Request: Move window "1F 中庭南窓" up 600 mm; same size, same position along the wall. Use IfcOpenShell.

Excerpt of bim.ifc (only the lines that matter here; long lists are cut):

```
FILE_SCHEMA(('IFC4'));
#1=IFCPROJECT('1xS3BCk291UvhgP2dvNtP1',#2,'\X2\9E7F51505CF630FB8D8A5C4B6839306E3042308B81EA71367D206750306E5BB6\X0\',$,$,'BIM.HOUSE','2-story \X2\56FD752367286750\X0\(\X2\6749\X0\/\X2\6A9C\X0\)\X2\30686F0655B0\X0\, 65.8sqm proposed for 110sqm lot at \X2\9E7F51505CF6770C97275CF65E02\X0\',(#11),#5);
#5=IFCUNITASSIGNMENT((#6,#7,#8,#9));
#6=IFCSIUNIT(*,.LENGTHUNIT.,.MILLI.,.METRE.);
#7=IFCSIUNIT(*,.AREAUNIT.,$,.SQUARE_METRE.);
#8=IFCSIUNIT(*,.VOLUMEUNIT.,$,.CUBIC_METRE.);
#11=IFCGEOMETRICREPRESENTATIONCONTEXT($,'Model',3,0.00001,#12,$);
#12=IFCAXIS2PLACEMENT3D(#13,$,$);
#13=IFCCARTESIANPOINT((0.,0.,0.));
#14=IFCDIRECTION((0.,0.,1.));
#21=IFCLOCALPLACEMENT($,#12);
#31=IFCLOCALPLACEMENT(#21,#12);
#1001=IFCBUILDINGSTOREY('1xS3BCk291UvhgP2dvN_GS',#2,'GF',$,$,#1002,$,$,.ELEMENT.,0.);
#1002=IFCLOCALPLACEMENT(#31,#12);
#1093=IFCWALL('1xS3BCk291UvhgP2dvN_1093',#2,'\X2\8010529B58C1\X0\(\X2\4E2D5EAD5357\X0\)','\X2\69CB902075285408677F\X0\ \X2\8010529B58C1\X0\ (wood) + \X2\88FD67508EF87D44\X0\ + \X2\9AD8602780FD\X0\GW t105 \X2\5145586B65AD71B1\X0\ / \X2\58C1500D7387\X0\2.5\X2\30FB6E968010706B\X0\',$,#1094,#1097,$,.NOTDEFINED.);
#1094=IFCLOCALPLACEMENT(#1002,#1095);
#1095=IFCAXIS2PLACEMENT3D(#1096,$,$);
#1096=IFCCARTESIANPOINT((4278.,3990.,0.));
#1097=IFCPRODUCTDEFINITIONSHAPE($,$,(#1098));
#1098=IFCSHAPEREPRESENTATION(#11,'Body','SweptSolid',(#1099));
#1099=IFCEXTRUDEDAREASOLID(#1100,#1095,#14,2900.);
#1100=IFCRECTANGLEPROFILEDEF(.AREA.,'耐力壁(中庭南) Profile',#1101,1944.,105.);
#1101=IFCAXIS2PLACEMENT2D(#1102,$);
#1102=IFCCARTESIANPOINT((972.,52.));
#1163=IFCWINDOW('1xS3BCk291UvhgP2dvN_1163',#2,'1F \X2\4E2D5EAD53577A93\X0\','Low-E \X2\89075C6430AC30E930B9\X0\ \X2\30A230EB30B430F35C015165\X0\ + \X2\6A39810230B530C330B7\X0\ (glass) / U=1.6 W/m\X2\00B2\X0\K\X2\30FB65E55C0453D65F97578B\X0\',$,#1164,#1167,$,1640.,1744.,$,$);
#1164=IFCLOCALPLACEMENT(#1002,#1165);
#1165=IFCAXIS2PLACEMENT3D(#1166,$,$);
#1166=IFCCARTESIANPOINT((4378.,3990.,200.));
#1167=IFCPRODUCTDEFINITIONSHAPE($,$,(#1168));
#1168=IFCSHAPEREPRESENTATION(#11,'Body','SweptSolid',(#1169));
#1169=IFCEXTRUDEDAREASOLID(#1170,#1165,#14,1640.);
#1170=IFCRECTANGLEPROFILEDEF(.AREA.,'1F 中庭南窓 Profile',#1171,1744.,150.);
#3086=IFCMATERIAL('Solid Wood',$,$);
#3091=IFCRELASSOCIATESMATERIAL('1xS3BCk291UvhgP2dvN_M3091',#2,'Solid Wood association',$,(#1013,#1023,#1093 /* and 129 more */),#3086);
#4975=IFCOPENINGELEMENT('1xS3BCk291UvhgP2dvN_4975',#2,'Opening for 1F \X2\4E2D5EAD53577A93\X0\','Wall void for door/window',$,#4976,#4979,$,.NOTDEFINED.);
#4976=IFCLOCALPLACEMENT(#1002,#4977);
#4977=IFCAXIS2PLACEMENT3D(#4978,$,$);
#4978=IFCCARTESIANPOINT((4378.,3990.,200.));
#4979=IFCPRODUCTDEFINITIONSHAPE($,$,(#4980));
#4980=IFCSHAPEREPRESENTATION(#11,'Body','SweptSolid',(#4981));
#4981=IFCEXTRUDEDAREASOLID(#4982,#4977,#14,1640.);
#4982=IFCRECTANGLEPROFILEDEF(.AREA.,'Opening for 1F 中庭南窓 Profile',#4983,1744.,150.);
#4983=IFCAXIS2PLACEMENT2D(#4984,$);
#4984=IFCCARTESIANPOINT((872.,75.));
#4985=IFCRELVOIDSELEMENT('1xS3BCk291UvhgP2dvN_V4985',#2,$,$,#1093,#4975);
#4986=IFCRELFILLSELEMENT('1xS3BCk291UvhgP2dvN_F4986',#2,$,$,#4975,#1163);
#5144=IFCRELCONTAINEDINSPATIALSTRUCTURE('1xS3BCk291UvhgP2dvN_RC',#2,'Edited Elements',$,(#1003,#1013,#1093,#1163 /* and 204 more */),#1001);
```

```python
import numpy as np
import ifcopenshell
import ifcopenshell.api.geometry
import ifcopenshell.util.placement
import ifcopenshell.util.unit

model = ifcopenshell.open("bim.ifc")
unit_scale = ifcopenshell.util.unit.calculate_unit_scale(model)

window = model.by_id(1163)
opening = window.FillsVoids[0].RelatingOpeningElement
dz = 0.6 / unit_scale

shift = np.array([0.0, 0.0, dz])
# The window is not placed relative to its opening, so move both.
for product in (opening, window):
    matrix = ifcopenshell.util.placement.get_local_placement(product.ObjectPlacement)
    matrix[:3, 3] += shift
    ifcopenshell.api.geometry.edit_object_placement(model, product=product, matrix=matrix, is_si=False)

print(f"moved by {dz * unit_scale:+.3f} m")

model.write("bim_updated.ifc")
```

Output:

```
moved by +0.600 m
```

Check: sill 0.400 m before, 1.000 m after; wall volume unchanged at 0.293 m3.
